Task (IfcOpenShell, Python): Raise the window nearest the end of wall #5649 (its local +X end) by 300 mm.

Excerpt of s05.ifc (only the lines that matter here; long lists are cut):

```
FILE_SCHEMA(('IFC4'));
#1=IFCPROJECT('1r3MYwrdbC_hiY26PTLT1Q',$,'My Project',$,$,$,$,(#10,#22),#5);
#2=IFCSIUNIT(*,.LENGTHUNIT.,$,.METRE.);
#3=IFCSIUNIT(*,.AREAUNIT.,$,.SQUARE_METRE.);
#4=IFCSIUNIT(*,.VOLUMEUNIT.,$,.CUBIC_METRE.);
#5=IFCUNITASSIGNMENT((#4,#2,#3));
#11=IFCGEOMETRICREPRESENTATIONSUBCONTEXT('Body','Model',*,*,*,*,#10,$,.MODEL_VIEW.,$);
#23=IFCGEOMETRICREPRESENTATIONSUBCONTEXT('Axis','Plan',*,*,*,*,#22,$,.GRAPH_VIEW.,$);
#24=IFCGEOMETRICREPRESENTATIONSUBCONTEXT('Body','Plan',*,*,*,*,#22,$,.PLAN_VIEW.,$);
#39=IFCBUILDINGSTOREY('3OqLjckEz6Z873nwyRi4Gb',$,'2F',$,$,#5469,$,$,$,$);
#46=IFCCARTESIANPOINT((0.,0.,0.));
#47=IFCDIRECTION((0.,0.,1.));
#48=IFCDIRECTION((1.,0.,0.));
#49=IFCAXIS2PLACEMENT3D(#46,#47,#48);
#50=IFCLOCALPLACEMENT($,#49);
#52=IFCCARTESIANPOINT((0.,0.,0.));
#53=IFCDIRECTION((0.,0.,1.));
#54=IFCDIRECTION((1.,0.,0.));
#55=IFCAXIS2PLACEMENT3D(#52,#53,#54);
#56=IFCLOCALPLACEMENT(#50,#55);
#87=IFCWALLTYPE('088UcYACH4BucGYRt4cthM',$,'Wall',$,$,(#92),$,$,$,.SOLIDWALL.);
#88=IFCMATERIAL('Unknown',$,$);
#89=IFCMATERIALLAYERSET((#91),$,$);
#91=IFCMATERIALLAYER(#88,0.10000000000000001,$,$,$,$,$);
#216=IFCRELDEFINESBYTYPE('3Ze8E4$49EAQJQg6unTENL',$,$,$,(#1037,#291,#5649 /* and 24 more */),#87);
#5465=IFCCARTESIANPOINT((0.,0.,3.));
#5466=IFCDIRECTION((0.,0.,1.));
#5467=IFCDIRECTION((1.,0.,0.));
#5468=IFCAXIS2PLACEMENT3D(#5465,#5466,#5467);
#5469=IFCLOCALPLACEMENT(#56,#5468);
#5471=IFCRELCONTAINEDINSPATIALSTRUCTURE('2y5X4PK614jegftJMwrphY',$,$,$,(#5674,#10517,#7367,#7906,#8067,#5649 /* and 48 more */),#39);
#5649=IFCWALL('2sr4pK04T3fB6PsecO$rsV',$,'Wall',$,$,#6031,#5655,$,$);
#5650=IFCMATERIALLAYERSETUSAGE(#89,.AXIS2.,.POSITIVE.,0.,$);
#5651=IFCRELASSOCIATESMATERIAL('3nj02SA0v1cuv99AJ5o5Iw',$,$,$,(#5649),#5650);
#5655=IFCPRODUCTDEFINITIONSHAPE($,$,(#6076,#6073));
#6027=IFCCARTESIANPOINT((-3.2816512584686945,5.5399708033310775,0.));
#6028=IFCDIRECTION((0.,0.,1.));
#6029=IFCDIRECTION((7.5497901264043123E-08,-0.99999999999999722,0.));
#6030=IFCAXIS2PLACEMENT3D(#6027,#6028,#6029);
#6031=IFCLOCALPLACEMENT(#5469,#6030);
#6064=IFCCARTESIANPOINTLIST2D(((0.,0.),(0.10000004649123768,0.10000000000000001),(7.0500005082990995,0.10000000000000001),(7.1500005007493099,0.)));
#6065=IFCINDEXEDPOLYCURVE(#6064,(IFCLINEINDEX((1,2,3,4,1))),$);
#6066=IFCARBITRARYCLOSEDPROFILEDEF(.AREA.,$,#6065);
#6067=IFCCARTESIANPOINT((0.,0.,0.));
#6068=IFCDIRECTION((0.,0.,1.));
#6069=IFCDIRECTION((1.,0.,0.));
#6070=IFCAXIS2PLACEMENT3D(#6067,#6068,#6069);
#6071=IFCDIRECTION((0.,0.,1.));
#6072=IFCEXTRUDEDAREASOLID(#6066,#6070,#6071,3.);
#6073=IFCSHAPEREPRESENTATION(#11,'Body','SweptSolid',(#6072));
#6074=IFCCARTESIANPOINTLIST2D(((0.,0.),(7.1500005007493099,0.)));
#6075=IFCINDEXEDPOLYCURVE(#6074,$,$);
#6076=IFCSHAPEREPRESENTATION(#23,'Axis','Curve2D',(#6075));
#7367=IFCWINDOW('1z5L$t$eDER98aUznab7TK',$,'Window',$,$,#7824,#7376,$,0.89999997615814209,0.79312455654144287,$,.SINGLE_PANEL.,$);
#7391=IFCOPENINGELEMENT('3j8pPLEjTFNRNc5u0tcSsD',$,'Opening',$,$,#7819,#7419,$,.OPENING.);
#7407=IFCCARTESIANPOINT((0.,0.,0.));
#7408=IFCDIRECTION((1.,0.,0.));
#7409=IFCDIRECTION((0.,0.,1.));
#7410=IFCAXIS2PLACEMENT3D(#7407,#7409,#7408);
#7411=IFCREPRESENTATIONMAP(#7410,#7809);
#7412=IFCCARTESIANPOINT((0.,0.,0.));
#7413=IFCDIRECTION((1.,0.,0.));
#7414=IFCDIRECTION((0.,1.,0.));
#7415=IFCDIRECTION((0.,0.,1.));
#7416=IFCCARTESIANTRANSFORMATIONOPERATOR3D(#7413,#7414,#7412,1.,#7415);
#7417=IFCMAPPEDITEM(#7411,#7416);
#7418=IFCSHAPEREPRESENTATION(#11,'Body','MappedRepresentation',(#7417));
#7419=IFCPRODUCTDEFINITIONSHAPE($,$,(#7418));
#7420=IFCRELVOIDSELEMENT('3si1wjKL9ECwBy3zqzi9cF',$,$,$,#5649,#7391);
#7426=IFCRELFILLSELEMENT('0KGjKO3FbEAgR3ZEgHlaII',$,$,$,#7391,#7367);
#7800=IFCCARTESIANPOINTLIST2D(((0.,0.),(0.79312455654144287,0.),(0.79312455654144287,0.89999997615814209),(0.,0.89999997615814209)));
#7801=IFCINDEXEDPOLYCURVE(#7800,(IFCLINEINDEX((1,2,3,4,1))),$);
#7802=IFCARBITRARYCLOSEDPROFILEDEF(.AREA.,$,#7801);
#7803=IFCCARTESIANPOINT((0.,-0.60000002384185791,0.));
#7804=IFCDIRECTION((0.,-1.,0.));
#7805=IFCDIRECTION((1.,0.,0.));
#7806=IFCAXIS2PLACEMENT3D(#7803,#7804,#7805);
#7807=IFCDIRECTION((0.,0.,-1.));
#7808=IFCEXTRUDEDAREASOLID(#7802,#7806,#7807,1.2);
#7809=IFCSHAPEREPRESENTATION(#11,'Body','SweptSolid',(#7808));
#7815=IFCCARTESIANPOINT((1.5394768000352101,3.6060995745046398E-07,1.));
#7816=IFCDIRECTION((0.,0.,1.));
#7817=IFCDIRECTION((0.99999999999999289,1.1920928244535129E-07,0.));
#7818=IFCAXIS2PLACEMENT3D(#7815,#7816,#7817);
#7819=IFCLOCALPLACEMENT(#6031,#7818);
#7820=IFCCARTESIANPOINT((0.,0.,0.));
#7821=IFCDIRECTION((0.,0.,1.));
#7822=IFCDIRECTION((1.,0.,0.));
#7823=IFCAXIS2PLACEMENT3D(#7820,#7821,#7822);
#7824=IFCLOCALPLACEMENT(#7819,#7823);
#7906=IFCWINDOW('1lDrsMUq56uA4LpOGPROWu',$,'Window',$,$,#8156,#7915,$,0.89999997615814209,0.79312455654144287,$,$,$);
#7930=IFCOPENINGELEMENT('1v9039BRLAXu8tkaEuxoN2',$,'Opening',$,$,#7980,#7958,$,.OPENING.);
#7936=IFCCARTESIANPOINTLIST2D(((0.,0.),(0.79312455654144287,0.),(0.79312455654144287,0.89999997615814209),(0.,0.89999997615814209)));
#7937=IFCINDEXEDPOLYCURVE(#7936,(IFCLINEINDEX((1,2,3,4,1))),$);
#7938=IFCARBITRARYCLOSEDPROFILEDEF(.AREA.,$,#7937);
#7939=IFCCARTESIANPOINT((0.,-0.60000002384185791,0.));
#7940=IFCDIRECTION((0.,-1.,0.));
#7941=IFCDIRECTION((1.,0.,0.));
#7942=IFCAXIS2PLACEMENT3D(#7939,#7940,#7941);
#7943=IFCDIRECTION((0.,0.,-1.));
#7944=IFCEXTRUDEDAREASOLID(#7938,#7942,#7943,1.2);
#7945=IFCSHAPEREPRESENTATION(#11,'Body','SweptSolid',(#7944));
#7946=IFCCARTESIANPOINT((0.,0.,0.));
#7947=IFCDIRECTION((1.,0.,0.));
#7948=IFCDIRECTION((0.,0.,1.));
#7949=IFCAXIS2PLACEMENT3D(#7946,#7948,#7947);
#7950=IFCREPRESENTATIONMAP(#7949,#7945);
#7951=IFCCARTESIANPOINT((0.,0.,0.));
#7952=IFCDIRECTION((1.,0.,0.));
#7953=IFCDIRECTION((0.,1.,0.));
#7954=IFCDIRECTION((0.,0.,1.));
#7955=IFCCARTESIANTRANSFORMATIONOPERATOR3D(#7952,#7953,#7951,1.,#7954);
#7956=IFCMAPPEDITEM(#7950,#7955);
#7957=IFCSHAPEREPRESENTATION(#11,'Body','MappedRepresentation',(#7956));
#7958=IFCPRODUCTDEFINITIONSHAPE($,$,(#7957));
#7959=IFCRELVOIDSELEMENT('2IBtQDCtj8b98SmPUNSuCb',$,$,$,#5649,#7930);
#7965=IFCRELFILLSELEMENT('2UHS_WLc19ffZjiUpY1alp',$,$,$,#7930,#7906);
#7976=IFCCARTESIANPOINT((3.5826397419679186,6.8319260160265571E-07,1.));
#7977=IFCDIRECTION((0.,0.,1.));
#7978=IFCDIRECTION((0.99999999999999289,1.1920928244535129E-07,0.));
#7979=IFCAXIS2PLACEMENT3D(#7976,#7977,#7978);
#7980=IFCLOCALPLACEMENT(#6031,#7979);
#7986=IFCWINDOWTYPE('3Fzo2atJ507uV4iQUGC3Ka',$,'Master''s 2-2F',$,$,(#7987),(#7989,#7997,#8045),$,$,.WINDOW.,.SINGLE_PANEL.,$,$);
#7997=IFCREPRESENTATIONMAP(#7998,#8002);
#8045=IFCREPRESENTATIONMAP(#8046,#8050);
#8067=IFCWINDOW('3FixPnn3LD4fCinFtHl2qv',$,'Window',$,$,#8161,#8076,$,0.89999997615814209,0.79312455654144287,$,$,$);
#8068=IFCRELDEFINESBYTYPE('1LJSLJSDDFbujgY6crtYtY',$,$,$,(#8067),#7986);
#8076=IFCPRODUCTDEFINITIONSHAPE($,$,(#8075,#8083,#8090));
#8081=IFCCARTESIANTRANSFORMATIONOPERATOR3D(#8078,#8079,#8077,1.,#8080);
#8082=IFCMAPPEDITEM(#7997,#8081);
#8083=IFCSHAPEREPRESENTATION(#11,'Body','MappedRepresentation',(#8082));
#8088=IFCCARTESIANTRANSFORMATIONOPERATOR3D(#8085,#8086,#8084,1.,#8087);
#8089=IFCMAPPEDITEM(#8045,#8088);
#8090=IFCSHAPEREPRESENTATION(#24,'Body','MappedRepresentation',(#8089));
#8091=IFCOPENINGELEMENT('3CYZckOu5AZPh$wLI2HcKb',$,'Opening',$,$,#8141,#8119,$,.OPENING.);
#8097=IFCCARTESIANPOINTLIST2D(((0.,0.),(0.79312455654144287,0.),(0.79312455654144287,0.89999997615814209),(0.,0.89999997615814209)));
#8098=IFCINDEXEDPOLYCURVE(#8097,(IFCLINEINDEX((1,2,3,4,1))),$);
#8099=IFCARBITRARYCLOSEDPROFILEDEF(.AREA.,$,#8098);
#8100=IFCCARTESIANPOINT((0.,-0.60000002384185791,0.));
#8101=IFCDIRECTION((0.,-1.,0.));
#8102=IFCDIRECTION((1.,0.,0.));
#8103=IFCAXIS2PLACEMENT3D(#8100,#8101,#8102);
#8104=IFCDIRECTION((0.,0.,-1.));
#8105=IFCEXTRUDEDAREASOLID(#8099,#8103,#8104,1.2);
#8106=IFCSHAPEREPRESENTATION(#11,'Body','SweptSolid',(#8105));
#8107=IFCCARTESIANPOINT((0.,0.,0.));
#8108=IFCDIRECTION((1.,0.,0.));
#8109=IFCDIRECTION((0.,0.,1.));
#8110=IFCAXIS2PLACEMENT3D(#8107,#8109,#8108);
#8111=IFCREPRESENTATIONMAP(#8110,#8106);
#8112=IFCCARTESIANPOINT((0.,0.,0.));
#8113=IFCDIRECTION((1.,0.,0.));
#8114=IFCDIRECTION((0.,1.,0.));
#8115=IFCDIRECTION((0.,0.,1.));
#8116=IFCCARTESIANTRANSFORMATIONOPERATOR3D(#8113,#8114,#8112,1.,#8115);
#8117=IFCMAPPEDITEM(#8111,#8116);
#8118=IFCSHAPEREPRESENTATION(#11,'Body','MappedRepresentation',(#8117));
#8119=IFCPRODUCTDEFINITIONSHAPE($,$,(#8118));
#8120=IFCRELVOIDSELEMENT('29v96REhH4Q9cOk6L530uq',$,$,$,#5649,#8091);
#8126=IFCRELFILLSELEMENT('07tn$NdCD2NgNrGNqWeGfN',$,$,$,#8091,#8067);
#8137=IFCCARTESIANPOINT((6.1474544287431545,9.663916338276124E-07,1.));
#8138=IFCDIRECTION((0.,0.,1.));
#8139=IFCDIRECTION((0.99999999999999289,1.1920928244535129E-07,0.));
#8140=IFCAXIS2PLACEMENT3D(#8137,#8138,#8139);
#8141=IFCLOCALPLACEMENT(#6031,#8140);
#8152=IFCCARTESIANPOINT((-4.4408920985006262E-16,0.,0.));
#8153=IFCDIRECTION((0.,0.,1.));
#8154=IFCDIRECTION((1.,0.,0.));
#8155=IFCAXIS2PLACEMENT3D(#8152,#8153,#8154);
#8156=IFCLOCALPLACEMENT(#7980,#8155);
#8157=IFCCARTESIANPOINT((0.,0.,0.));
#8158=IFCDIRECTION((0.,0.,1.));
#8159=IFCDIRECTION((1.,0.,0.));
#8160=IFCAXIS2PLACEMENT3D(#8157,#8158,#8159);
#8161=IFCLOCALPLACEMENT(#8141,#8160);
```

```python
import numpy as np
import ifcopenshell
import ifcopenshell.api.geometry
import ifcopenshell.util.placement
import ifcopenshell.util.unit

model = ifcopenshell.open("s05.ifc")
unit_scale = ifcopenshell.util.unit.calculate_unit_scale(model)

window = model.by_guid("3FixPnn3LD4fCinFtHl2qv")
opening = window.FillsVoids[0].RelatingOpeningElement
dz = 0.3 / unit_scale

shift = np.array([0.0, 0.0, dz])
# The window is placed relative to its opening, so it follows when the opening moves.
matrix = ifcopenshell.util.placement.get_local_placement(opening.ObjectPlacement)
matrix[:3, 3] += shift
ifcopenshell.api.geometry.edit_object_placement(
    model, product=opening, matrix=matrix, is_si=False, should_transform_children=True
)

print(f"moved by {dz * unit_scale:+.3f} m")

model.write("s05_edited.ifc")
```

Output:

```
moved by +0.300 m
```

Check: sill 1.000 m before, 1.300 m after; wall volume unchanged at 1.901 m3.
